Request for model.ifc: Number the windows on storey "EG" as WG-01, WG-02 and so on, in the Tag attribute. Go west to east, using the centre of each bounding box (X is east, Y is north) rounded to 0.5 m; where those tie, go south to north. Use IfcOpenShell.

First a look at what the model holds.

```python
import ifcopenshell
import ifcopenshell.util.element
import ifcopenshell.util.placement

model = ifcopenshell.open("model.ifc")
print(model.schema)
storey = next(s for s in model.by_type("IfcBuildingStorey") if s.Name == "EG")
windows = [e for e in ifcopenshell.util.element.get_decomposition(storey) if e.is_a("IfcWindow")]
for e in sorted(windows, key=lambda e: e.id()):
    origin = ifcopenshell.util.placement.get_local_placement(e.ObjectPlacement)[:3, 3]
    print(e.id(), e.Tag, e.Name, origin.round(2) + 0.0, sep=" | ")
```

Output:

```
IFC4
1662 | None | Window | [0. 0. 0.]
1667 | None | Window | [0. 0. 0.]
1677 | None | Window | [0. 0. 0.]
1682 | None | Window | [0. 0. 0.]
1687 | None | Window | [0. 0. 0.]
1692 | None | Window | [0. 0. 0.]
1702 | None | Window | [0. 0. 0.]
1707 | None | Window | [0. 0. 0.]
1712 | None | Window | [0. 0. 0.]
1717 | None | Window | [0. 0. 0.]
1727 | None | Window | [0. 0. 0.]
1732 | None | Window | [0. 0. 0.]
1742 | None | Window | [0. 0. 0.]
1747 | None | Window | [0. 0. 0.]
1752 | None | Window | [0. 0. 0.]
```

```python
import ifcopenshell
import ifcopenshell.geom
import ifcopenshell.util.element
import ifcopenshell.util.shape

model = ifcopenshell.open("model.ifc")
settings = ifcopenshell.geom.settings()
settings.set("use-world-coords", True)


def centre(element):
    shape = ifcopenshell.geom.create_shape(settings, element)
    return ifcopenshell.util.shape.get_bbox_centroid(shape.geometry)


storey = next(s for s in model.by_type("IfcBuildingStorey") if s.Name == "EG")
windows = [e for e in ifcopenshell.util.element.get_decomposition(storey) if e.is_a("IfcWindow")]

# Insertion points can sit at a corner or the storey origin, so sort by the geometry (in metres).
centres = {e: centre(e) for e in windows}
windows.sort(key=lambda e: (round(centres[e][0] / 0.5), centres[e][1]))

for i, e in enumerate(windows, start=1):
    number = f"WG-{i:02d}"
    e.Tag = number
    print(e.id(), number)

model.write("model_rev.ifc")
```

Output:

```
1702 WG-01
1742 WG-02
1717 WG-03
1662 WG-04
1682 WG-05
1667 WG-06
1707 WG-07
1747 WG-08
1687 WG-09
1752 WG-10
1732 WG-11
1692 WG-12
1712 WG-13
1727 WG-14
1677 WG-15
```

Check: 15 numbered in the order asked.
